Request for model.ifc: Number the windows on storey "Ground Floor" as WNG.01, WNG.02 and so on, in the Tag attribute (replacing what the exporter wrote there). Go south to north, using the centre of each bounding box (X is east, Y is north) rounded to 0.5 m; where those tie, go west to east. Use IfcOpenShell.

First a look at what the model holds.

```python
import ifcopenshell
import ifcopenshell.util.element
import ifcopenshell.util.placement

model = ifcopenshell.open("model.ifc")
print(model.schema)
storey = next(s for s in model.by_type("IfcBuildingStorey") if s.Name == "Ground Floor")
windows = [e for e in ifcopenshell.util.element.get_decomposition(storey) if e.is_a("IfcWindow")]
for e in sorted(windows, key=lambda e: e.id()):
    origin = ifcopenshell.util.placement.get_local_placement(e.ObjectPlacement)[:3, 3]
    print(e.id(), e.Tag, e.Name, origin.round(2) + 0.0, sep=" | ")
```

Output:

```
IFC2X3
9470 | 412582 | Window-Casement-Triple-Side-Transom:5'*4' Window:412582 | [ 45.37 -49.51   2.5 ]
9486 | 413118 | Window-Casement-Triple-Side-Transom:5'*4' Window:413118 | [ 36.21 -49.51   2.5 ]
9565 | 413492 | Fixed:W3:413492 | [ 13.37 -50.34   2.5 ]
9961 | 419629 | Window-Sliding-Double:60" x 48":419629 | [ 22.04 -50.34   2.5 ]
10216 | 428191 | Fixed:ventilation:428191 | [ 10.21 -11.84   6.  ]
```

```python
import ifcopenshell
import ifcopenshell.geom
import ifcopenshell.util.element
import ifcopenshell.util.shape

model = ifcopenshell.open("model.ifc")
settings = ifcopenshell.geom.settings()
settings.set("use-world-coords", True)


def centre(element):
    shape = ifcopenshell.geom.create_shape(settings, element)
    return ifcopenshell.util.shape.get_bbox_centroid(shape.geometry)


storey = next(s for s in model.by_type("IfcBuildingStorey") if s.Name == "Ground Floor")
windows = [e for e in ifcopenshell.util.element.get_decomposition(storey) if e.is_a("IfcWindow")]

# Insertion points can sit at a corner or the storey origin, so sort by the geometry (in metres).
centres = {e: centre(e) for e in windows}
windows.sort(key=lambda e: (round(centres[e][1] / 0.5), centres[e][0]))

for i, e in enumerate(windows, start=1):
    number = f"WNG.{i:02d}"
    e.Tag = number
    print(e.id(), number)

model.write("model_v2.ifc")
```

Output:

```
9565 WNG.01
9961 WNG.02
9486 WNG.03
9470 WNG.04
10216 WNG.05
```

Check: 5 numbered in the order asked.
